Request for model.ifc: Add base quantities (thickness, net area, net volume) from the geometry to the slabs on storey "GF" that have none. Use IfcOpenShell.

First a look at what the model holds.

```python
import ifcopenshell
import ifcopenshell.util.element
import ifcopenshell.util.unit

model = ifcopenshell.open("model.ifc")
print(model.schema)
for unit_type in ("LENGTHUNIT", "AREAUNIT", "VOLUMEUNIT"):
    print(unit_type, ifcopenshell.util.unit.calculate_unit_scale(model, unit_type))
storey = next(s for s in model.by_type("IfcBuildingStorey") if s.Name == "GF")
slabs = [e for e in ifcopenshell.util.element.get_decomposition(storey) if e.is_a("IfcSlab")]
for e in sorted(slabs, key=lambda e: e.id()):
    print(e.id(), e.is_a(), e.Name, list(ifcopenshell.util.element.get_psets(e, qtos_only=True)), sep=" | ")
```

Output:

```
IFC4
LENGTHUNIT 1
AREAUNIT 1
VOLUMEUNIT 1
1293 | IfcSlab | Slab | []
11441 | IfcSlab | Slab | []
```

```python
import ifcopenshell
import ifcopenshell.api.pset
import ifcopenshell.geom
import ifcopenshell.util.element
import ifcopenshell.util.shape
import ifcopenshell.util.unit

model = ifcopenshell.open("model.ifc")
unit_scale = ifcopenshell.util.unit.calculate_unit_scale(model)
area_scale = ifcopenshell.util.unit.calculate_unit_scale(model, "AREAUNIT")
volume_scale = ifcopenshell.util.unit.calculate_unit_scale(model, "VOLUMEUNIT")
settings = ifcopenshell.geom.settings()

storey = next(s for s in model.by_type("IfcBuildingStorey") if s.Name == "GF")
slabs = [e for e in ifcopenshell.util.element.get_decomposition(storey) if e.is_a("IfcSlab")]

for e in sorted(slabs, key=lambda e: e.id()):
    if ifcopenshell.util.element.get_psets(e, qtos_only=True, should_inherit=False):
        continue
    # Geometry comes back in metres, in the element's own axes.
    shape = ifcopenshell.geom.create_shape(settings, e)
    values = {
        "Width": ifcopenshell.util.shape.get_z(shape.geometry) / unit_scale,
        "NetArea": ifcopenshell.util.shape.get_footprint_area(shape.geometry) / area_scale,
        "NetVolume": ifcopenshell.util.shape.get_volume(shape.geometry) / volume_scale,
    }
    qto = ifcopenshell.api.pset.add_qto(model, product=e, name="Qto_SlabBaseQuantities")
    ifcopenshell.api.pset.edit_qto(model, qto=qto, properties=values)
    print(e.id(), {k: round(v, 3) for k, v in values.items()})

model.write("model-out.ifc")
```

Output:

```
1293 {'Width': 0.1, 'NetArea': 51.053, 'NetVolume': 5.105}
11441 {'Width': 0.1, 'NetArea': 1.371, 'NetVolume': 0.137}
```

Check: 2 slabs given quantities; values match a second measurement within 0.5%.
